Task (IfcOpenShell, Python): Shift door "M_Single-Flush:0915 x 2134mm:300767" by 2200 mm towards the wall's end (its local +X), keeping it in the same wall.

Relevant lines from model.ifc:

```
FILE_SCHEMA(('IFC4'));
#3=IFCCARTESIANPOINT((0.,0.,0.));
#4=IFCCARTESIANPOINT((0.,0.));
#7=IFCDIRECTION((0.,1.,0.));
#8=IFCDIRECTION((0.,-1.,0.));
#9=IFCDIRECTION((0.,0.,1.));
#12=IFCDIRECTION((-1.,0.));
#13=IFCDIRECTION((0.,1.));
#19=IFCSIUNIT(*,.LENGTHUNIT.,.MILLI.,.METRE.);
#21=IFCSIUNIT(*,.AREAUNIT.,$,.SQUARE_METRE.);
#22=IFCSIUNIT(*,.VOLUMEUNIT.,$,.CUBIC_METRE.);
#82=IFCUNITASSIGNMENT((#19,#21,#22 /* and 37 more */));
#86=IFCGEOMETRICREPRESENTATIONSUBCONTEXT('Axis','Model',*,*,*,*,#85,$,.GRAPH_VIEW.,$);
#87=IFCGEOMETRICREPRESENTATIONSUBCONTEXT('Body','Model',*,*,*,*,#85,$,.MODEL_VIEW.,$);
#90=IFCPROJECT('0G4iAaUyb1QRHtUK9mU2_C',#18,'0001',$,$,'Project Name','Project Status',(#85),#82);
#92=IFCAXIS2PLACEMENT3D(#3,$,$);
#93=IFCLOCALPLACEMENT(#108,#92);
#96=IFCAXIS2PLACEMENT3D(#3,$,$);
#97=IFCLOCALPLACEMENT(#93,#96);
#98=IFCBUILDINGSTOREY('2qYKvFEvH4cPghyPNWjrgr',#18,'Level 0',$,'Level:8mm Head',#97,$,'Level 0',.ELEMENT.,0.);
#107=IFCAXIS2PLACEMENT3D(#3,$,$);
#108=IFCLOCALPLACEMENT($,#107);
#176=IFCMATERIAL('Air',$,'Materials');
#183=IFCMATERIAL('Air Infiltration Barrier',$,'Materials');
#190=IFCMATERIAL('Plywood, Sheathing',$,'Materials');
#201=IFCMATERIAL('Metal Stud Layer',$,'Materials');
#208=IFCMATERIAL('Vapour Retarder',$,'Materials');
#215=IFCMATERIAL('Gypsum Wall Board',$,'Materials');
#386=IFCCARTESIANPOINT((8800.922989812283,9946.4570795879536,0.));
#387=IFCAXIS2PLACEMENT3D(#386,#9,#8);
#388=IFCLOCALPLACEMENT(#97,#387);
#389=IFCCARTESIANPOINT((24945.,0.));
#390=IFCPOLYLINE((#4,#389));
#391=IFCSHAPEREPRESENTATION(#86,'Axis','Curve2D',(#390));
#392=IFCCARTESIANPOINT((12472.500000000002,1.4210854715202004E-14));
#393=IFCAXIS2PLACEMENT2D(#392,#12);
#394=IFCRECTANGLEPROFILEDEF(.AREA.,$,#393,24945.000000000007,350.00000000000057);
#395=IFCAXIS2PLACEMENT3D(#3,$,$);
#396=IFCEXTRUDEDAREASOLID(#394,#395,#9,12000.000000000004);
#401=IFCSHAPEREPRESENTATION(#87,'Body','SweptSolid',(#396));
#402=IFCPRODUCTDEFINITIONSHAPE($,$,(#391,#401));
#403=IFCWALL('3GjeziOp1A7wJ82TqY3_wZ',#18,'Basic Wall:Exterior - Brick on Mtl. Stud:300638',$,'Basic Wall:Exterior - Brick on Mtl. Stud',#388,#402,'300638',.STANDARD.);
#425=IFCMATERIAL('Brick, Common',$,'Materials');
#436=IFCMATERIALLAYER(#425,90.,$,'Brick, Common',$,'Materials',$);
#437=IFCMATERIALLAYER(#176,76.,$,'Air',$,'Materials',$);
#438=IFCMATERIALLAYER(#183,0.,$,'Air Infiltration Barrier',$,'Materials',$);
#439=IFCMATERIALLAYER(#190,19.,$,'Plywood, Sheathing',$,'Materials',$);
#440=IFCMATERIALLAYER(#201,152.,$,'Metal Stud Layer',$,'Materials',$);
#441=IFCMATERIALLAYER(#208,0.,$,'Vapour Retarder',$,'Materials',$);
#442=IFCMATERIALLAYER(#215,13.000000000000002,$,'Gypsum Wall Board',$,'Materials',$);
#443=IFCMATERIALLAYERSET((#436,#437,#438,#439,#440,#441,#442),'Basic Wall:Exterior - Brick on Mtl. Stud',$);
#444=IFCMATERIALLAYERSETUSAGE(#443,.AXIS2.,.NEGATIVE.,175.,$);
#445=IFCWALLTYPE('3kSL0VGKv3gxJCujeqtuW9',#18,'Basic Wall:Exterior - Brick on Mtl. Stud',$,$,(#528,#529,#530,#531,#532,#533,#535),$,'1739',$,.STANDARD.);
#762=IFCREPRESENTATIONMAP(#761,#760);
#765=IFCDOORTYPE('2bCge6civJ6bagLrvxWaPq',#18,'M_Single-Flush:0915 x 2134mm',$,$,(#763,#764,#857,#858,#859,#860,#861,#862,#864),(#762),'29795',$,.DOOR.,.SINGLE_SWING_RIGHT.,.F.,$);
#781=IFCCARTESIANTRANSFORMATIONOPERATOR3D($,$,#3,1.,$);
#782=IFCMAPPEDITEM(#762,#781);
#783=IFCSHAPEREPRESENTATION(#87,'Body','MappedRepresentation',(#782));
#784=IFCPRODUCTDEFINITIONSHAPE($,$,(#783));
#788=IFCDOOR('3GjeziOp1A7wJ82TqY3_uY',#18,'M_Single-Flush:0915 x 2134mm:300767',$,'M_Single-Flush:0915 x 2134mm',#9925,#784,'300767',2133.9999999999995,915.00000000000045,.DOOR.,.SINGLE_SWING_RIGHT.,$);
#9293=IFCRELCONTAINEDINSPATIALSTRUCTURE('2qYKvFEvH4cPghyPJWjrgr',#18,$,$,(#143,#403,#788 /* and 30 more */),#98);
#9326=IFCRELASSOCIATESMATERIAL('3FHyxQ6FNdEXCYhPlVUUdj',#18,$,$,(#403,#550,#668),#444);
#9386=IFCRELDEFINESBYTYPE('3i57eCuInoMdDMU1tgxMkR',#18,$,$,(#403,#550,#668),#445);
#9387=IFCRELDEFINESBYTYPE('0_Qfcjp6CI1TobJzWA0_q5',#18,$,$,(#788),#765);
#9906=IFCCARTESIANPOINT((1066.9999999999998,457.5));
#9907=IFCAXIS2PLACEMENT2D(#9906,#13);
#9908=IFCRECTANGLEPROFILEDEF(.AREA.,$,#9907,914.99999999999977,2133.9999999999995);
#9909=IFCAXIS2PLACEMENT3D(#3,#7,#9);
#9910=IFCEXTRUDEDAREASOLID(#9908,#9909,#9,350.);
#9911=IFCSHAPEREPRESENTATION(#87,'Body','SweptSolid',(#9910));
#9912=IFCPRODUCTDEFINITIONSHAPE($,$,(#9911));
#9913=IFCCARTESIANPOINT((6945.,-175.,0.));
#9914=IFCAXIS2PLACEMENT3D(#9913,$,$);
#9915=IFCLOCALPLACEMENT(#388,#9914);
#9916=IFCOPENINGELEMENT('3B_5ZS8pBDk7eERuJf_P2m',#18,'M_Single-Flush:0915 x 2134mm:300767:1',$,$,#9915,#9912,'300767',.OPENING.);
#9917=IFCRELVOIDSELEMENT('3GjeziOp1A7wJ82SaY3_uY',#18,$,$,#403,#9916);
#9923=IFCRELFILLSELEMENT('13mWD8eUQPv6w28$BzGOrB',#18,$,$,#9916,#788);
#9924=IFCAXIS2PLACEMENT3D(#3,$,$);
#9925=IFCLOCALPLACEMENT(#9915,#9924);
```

```python
import ifcopenshell
import ifcopenshell.api.geometry
import ifcopenshell.util.placement

model = ifcopenshell.open("model.ifc")

door = model.by_id(788)
opening = door.FillsVoids[0].RelatingOpeningElement
wall = opening.VoidsElements[0].RelatingBuildingElement

wall_matrix = ifcopenshell.util.placement.get_local_placement(wall.ObjectPlacement)
shift = wall_matrix[:3, 0] * 2200.0
before = ifcopenshell.util.placement.get_local_placement(door.ObjectPlacement)[:3, 3].copy()

# The door is placed relative to its opening, so it follows when the opening moves.
matrix = ifcopenshell.util.placement.get_local_placement(opening.ObjectPlacement)
matrix[:3, 3] += shift
ifcopenshell.api.geometry.edit_object_placement(
    model, product=opening, matrix=matrix, is_si=False, should_transform_children=True
)

after = ifcopenshell.util.placement.get_local_placement(door.ObjectPlacement)[:3, 3]
print("door moved by", (after - before).round(3) + 0.0)

model.write("model-out.ifc")
```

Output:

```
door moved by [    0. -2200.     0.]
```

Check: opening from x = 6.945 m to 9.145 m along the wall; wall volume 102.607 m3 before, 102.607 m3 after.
